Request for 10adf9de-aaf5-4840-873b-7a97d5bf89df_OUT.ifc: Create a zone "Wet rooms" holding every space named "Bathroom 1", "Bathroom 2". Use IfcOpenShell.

First a look at what the model holds.

```python
import ifcopenshell

model = ifcopenshell.open("10adf9de-aaf5-4840-873b-7a97d5bf89df_OUT.ifc")
print(model.schema)
seen = {}
for space in model.by_type("IfcSpace"):
    seen[space.LongName] = seen.get(space.LongName, 0) + 1
for name, count in sorted(seen.items(), key=str):
    print(count, "x", name)
print("zones:", [z.Name for z in model.by_type("IfcZone")][:20])
```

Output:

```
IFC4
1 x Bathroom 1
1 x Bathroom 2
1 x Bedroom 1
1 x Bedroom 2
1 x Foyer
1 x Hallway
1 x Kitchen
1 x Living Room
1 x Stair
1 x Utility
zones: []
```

```python
import ifcopenshell
import ifcopenshell.api.group
import ifcopenshell.api.root

model = ifcopenshell.open("10adf9de-aaf5-4840-873b-7a97d5bf89df_OUT.ifc")

names = {"Bathroom 1", "Bathroom 2"}
spaces = [s for s in model.by_type("IfcSpace") if s.LongName in names]

zone = ifcopenshell.api.root.create_entity(model, ifc_class="IfcZone", name="Wet rooms")
ifcopenshell.api.group.assign_group(model, products=spaces, group=zone)
print(len(spaces), "spaces in", zone.Name)

model.write("10adf9de-aaf5-4840-873b-7a97d5bf89df_OUT-out.ifc")
```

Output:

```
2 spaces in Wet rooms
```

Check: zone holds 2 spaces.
